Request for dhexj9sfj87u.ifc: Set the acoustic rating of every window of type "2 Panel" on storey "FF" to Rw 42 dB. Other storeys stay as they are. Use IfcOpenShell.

First a look at what the model holds.

```python
import ifcopenshell
import ifcopenshell.util.element

model = ifcopenshell.open("dhexj9sfj87u.ifc")
print(model.schema)
storey = next(s for s in model.by_type("IfcBuildingStorey") if s.Name == "FF")
windows = [e for e in ifcopenshell.util.element.get_decomposition(storey) if e.is_a("IfcWindow")]
seen = {}
for e in windows:
    element_type = ifcopenshell.util.element.get_type(e)
    key = (element_type.Name if element_type != e and element_type else None, ifcopenshell.util.element.get_pset(e, "Pset_WindowCommon", "AcousticRating"))
    seen[key] = seen.get(key, 0) + 1
for (name, value), count in sorted(seen.items(), key=str):
    print(count, "x", name, "|", value)
```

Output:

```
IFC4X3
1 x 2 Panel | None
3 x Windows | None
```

```python
import ifcopenshell
import ifcopenshell.api.pset
import ifcopenshell.util.element

model = ifcopenshell.open("dhexj9sfj87u.ifc")

storey = next(s for s in model.by_type("IfcBuildingStorey") if s.Name == "FF")
windows = [e for e in ifcopenshell.util.element.get_decomposition(storey) if e.is_a("IfcWindow")]

count = 0
for e in windows:
    element_type = ifcopenshell.util.element.get_type(e)
    if element_type in (None, e) or element_type.Name != "2 Panel":
        continue
    # add_pset returns the element's existing set when there is one.
    pset = ifcopenshell.api.pset.add_pset(model, product=e, name="Pset_WindowCommon")
    ifcopenshell.api.pset.edit_pset(model, pset=pset, properties={"AcousticRating": "Rw 42 dB"})
    count += 1

print(count, "windows updated")

model.write("dhexj9sfj87u_edited.ifc")
```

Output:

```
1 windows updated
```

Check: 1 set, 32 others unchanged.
